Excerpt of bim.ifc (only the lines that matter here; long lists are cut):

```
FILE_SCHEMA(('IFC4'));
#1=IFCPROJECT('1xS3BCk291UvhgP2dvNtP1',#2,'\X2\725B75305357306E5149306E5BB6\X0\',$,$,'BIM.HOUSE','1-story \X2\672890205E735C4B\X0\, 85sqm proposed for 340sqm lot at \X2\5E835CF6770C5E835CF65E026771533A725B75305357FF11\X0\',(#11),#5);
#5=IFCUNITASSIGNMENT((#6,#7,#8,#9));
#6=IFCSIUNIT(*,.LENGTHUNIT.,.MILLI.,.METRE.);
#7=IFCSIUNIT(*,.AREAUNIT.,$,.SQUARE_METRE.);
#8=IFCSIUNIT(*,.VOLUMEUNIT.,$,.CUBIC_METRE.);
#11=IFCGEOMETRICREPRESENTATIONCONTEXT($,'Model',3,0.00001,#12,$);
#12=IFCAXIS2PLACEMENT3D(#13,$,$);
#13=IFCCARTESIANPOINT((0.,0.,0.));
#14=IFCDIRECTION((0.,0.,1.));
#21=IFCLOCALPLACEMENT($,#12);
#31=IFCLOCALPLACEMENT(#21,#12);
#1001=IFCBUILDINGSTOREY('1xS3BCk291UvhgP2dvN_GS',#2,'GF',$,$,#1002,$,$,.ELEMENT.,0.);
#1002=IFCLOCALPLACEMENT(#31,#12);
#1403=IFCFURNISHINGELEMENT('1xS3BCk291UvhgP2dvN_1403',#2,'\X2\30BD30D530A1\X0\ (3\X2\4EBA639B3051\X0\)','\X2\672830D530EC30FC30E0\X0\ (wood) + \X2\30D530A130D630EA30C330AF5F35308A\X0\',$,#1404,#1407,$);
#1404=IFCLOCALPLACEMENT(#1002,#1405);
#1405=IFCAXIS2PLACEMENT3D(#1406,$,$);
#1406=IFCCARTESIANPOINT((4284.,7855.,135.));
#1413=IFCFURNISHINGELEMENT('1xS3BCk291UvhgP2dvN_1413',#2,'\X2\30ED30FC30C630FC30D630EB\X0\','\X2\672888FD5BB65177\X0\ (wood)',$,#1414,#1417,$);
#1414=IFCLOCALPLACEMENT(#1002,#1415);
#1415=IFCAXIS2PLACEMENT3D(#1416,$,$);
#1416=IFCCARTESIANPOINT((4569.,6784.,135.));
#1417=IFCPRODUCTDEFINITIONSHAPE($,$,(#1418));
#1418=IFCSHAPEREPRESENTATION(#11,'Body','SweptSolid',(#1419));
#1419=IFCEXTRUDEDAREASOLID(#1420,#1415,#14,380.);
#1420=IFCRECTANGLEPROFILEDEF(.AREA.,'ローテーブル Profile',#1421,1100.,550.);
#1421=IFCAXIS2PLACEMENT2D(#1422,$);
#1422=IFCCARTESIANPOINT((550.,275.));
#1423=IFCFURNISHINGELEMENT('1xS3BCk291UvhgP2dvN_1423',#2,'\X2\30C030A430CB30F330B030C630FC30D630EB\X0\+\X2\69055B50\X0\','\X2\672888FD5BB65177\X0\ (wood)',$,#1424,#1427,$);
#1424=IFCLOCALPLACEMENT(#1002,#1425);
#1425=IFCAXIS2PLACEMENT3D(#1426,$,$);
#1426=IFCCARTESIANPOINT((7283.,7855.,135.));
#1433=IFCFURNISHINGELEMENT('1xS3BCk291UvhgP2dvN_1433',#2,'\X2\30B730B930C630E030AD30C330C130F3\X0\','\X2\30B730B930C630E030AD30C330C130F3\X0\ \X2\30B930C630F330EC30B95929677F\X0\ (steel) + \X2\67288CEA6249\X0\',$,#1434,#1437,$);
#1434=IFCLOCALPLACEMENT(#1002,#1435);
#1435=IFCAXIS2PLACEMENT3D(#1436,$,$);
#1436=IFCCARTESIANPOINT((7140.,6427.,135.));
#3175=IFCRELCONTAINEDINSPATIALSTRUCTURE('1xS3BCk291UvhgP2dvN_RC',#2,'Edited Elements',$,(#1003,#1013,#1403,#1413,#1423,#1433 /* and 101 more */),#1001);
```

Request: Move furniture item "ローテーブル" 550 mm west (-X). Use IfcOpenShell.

```python
import ifcopenshell
import ifcopenshell.api.geometry
import ifcopenshell.util.placement
import ifcopenshell.util.unit

model = ifcopenshell.open("bim.ifc")
unit_scale = ifcopenshell.util.unit.calculate_unit_scale(model)

item = model.by_id(1413)
matrix = ifcopenshell.util.placement.get_local_placement(item.ObjectPlacement)
matrix[0, 3] -= 0.55 / unit_scale
ifcopenshell.api.geometry.edit_object_placement(model, product=item, matrix=matrix, is_si=False)

print(ifcopenshell.util.placement.get_local_placement(item.ObjectPlacement).round(3) + 0.0)

model.write("bim_updated.ifc")
```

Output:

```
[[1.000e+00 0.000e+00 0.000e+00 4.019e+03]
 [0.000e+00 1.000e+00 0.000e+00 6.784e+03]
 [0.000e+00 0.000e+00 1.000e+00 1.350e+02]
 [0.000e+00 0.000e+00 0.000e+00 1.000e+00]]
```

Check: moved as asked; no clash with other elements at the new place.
